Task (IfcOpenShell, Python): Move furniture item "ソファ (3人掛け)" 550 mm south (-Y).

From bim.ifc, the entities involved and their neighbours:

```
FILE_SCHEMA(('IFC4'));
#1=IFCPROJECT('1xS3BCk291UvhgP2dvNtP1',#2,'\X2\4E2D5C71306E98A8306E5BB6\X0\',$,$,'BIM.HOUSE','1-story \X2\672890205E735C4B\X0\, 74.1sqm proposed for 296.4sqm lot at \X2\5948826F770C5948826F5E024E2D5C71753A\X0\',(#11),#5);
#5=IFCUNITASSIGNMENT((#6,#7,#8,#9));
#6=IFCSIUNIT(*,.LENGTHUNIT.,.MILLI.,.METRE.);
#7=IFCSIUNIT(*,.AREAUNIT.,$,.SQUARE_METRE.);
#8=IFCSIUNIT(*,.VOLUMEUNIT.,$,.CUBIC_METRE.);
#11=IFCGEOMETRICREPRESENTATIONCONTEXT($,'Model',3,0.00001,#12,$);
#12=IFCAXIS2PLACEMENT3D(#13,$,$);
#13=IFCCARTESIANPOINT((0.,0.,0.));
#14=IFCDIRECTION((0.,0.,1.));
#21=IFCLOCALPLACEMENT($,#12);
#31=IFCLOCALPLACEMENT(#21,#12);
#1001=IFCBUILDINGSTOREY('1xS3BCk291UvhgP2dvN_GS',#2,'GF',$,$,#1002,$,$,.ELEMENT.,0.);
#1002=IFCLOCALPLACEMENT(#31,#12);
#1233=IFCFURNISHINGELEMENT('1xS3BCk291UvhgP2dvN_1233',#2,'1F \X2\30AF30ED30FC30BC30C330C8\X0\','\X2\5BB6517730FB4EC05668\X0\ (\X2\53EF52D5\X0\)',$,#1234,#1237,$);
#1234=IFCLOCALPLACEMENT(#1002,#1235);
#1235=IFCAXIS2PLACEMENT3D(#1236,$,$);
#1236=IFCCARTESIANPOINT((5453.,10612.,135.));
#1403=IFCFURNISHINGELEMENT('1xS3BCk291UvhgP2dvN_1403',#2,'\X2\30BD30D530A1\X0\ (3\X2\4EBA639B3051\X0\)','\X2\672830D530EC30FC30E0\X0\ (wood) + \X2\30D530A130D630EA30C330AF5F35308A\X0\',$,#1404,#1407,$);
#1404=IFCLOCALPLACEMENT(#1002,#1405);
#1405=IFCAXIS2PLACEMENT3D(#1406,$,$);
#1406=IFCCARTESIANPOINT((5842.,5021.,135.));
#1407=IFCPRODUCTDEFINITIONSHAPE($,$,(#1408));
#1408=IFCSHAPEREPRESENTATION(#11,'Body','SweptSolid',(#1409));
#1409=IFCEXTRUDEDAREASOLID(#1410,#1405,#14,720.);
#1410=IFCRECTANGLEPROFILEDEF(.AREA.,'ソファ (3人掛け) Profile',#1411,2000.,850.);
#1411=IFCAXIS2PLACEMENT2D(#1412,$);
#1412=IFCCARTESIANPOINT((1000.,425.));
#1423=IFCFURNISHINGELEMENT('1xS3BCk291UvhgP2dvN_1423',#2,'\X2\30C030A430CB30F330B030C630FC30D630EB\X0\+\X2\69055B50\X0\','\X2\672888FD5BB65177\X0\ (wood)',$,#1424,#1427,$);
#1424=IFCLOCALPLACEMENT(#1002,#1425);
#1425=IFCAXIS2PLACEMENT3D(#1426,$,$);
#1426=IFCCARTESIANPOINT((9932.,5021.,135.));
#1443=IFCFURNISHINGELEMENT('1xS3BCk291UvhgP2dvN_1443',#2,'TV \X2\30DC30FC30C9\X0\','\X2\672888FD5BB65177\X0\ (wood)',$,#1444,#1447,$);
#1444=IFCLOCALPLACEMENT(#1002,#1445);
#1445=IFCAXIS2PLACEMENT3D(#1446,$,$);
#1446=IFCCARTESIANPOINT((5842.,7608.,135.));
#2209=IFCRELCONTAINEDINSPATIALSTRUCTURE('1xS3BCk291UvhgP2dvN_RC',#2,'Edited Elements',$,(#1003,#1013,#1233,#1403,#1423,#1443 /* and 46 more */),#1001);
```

```python
import ifcopenshell
import ifcopenshell.api.geometry
import ifcopenshell.util.placement
import ifcopenshell.util.unit

model = ifcopenshell.open("bim.ifc")
unit_scale = ifcopenshell.util.unit.calculate_unit_scale(model)

item = model.by_guid("1xS3BCk291UvhgP2dvN_1403")
matrix = ifcopenshell.util.placement.get_local_placement(item.ObjectPlacement)
matrix[1, 3] -= 0.55 / unit_scale
ifcopenshell.api.geometry.edit_object_placement(model, product=item, matrix=matrix, is_si=False)

print(ifcopenshell.util.placement.get_local_placement(item.ObjectPlacement).round(3) + 0.0)

model.write("bim_updated.ifc")
```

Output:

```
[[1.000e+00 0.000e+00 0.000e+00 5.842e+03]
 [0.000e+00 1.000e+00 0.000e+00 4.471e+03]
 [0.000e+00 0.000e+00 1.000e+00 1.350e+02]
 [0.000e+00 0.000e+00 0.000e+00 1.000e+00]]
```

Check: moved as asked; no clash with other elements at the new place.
